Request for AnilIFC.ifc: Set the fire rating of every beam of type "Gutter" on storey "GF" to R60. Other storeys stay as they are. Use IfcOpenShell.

First a look at what the model holds.

```python
import ifcopenshell
import ifcopenshell.util.element

model = ifcopenshell.open("AnilIFC.ifc")
print(model.schema)
storey = next(s for s in model.by_type("IfcBuildingStorey") if s.Name == "GF")
beams = [e for e in ifcopenshell.util.element.get_decomposition(storey) if e.is_a("IfcBeam")]
seen = {}
for e in beams:
    element_type = ifcopenshell.util.element.get_type(e)
    key = (element_type.Name if element_type != e and element_type else None, ifcopenshell.util.element.get_pset(e, "Pset_BeamCommon", "FireRating"))
    seen[key] = seen.get(key, 0) + 1
for (name, value), count in sorted(seen.items(), key=str):
    print(count, "x", name, "|", value)
```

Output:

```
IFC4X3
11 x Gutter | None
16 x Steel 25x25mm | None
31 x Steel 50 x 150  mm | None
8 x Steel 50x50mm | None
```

```python
import ifcopenshell
import ifcopenshell.api.pset
import ifcopenshell.util.element

model = ifcopenshell.open("AnilIFC.ifc")

storey = next(s for s in model.by_type("IfcBuildingStorey") if s.Name == "GF")
beams = [e for e in ifcopenshell.util.element.get_decomposition(storey) if e.is_a("IfcBeam")]

count = 0
for e in beams:
    element_type = ifcopenshell.util.element.get_type(e)
    if element_type in (None, e) or element_type.Name != "Gutter":
        continue
    # add_pset returns the element's existing set when there is one.
    pset = ifcopenshell.api.pset.add_pset(model, product=e, name="Pset_BeamCommon")
    ifcopenshell.api.pset.edit_pset(model, pset=pset, properties={"FireRating": "R60"})
    count += 1

print(count, "beams updated")

model.write("AnilIFC_v2.ifc")
```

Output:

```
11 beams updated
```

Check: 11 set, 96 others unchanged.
